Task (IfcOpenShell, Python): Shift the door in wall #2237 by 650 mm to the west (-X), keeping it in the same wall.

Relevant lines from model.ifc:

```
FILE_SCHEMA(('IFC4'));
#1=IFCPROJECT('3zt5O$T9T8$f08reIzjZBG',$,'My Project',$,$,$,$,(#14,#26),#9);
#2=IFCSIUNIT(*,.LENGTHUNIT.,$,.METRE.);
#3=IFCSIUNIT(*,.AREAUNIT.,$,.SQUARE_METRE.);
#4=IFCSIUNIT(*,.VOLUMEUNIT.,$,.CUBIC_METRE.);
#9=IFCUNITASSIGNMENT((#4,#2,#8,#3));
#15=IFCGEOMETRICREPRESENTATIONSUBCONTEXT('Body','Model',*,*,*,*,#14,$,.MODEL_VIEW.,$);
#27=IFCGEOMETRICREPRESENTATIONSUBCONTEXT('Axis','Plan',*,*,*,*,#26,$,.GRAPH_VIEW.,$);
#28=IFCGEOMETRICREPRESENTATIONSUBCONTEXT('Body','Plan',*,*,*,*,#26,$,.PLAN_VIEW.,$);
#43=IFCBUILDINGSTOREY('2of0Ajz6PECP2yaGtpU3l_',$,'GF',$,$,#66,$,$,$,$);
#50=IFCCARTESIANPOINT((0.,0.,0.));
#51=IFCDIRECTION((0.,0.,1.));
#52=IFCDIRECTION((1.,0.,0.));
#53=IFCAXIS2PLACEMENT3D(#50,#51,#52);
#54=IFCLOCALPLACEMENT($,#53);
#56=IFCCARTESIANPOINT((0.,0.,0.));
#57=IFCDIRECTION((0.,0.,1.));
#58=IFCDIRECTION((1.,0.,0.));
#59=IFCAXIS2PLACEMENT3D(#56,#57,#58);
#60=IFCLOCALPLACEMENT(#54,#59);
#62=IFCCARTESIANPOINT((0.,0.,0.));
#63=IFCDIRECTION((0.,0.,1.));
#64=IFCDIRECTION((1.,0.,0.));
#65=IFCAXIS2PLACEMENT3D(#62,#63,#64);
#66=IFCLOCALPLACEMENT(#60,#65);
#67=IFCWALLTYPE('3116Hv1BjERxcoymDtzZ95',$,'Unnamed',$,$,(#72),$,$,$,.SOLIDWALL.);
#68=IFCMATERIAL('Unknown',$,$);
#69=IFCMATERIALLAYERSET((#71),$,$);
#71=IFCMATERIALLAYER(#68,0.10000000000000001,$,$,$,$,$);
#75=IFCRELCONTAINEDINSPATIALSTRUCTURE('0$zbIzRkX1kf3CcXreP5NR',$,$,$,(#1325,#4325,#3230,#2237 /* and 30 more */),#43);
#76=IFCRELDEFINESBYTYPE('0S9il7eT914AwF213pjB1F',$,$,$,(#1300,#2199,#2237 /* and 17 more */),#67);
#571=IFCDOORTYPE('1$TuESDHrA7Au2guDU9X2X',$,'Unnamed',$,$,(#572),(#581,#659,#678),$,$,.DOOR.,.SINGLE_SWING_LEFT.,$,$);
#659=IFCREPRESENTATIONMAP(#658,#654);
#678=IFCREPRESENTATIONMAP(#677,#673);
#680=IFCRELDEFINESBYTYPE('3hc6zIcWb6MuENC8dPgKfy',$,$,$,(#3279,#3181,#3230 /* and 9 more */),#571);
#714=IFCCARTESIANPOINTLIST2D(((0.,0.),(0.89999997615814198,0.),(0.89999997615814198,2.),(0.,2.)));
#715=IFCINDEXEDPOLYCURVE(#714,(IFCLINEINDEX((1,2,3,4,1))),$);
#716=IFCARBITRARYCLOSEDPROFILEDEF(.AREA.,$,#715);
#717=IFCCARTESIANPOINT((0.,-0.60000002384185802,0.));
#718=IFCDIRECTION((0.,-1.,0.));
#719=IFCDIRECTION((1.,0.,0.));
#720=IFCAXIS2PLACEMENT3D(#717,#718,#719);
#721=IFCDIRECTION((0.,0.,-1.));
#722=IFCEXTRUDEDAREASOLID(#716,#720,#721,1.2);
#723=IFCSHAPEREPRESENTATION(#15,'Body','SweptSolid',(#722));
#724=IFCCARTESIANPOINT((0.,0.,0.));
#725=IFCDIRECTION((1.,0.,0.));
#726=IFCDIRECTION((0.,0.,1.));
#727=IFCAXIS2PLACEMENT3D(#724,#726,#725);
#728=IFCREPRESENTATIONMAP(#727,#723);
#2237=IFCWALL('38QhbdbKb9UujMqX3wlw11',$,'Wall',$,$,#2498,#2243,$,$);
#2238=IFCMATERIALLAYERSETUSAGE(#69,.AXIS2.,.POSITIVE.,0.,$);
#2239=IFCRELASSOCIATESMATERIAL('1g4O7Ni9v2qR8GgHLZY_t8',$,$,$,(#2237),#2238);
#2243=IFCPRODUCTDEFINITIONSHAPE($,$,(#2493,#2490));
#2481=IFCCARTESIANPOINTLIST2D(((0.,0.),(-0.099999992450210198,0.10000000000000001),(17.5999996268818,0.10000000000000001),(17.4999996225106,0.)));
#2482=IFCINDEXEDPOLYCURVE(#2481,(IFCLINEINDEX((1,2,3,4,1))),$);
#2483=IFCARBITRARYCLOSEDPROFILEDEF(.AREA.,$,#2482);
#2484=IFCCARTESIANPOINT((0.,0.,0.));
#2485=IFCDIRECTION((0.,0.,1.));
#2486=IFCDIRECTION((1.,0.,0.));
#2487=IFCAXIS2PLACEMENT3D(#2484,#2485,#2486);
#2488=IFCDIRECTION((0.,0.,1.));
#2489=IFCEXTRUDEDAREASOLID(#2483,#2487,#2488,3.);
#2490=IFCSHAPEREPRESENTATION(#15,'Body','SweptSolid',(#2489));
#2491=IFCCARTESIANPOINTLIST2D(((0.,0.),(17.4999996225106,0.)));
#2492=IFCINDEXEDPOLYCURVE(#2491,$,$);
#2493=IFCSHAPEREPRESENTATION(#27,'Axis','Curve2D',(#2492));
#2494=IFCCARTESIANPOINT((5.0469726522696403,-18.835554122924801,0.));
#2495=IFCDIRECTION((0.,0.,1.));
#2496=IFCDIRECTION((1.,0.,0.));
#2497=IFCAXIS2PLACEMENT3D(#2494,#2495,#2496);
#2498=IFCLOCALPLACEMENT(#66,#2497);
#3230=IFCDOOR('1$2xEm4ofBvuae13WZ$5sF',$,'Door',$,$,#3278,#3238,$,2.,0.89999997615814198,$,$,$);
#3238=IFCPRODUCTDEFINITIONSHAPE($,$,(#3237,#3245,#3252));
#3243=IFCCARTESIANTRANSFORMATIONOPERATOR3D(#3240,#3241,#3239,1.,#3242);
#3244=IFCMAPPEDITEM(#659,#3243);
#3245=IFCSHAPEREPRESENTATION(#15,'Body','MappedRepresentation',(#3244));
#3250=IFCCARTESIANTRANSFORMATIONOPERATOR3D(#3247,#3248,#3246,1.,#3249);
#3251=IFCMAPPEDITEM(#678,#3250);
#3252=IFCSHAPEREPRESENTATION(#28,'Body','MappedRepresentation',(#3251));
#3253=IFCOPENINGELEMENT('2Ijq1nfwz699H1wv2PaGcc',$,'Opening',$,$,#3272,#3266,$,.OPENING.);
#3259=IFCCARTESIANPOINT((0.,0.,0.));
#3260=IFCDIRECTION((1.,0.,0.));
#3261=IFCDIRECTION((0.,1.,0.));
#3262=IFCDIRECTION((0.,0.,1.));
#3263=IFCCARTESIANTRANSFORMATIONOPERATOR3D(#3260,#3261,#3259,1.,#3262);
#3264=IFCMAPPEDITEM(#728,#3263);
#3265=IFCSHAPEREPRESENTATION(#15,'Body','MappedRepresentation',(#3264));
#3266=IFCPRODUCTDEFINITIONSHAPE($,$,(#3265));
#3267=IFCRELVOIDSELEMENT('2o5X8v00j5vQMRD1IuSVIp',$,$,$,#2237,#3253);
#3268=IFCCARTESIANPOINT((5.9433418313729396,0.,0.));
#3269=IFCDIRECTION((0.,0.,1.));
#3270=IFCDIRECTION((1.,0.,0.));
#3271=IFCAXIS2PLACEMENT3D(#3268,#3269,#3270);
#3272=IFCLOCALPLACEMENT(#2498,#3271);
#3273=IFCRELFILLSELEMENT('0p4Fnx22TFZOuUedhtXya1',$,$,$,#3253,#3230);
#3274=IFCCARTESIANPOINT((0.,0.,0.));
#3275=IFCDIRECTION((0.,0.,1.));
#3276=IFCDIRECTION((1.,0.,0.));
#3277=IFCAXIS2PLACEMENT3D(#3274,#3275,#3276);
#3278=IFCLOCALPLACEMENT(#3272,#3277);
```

```python
import ifcopenshell
import ifcopenshell.api.geometry
import ifcopenshell.util.placement
import ifcopenshell.util.unit

model = ifcopenshell.open("model.ifc")
unit_scale = ifcopenshell.util.unit.calculate_unit_scale(model)

door = model.by_guid("1$2xEm4ofBvuae13WZ$5sF")
opening = door.FillsVoids[0].RelatingOpeningElement
wall = opening.VoidsElements[0].RelatingBuildingElement

wall_matrix = ifcopenshell.util.placement.get_local_placement(wall.ObjectPlacement)
shift = wall_matrix[:3, 0] * -0.65 / unit_scale
before = ifcopenshell.util.placement.get_local_placement(door.ObjectPlacement)[:3, 3].copy()

# The door is placed relative to its opening, so it follows when the opening moves.
matrix = ifcopenshell.util.placement.get_local_placement(opening.ObjectPlacement)
matrix[:3, 3] += shift
ifcopenshell.api.geometry.edit_object_placement(
    model, product=opening, matrix=matrix, is_si=False, should_transform_children=True
)

after = ifcopenshell.util.placement.get_local_placement(door.ObjectPlacement)[:3, 3]
print("door moved by", (after - before).round(3) + 0.0)

model.write("model_v2.ifc")
```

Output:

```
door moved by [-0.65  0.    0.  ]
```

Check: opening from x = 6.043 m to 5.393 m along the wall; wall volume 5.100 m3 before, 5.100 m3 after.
